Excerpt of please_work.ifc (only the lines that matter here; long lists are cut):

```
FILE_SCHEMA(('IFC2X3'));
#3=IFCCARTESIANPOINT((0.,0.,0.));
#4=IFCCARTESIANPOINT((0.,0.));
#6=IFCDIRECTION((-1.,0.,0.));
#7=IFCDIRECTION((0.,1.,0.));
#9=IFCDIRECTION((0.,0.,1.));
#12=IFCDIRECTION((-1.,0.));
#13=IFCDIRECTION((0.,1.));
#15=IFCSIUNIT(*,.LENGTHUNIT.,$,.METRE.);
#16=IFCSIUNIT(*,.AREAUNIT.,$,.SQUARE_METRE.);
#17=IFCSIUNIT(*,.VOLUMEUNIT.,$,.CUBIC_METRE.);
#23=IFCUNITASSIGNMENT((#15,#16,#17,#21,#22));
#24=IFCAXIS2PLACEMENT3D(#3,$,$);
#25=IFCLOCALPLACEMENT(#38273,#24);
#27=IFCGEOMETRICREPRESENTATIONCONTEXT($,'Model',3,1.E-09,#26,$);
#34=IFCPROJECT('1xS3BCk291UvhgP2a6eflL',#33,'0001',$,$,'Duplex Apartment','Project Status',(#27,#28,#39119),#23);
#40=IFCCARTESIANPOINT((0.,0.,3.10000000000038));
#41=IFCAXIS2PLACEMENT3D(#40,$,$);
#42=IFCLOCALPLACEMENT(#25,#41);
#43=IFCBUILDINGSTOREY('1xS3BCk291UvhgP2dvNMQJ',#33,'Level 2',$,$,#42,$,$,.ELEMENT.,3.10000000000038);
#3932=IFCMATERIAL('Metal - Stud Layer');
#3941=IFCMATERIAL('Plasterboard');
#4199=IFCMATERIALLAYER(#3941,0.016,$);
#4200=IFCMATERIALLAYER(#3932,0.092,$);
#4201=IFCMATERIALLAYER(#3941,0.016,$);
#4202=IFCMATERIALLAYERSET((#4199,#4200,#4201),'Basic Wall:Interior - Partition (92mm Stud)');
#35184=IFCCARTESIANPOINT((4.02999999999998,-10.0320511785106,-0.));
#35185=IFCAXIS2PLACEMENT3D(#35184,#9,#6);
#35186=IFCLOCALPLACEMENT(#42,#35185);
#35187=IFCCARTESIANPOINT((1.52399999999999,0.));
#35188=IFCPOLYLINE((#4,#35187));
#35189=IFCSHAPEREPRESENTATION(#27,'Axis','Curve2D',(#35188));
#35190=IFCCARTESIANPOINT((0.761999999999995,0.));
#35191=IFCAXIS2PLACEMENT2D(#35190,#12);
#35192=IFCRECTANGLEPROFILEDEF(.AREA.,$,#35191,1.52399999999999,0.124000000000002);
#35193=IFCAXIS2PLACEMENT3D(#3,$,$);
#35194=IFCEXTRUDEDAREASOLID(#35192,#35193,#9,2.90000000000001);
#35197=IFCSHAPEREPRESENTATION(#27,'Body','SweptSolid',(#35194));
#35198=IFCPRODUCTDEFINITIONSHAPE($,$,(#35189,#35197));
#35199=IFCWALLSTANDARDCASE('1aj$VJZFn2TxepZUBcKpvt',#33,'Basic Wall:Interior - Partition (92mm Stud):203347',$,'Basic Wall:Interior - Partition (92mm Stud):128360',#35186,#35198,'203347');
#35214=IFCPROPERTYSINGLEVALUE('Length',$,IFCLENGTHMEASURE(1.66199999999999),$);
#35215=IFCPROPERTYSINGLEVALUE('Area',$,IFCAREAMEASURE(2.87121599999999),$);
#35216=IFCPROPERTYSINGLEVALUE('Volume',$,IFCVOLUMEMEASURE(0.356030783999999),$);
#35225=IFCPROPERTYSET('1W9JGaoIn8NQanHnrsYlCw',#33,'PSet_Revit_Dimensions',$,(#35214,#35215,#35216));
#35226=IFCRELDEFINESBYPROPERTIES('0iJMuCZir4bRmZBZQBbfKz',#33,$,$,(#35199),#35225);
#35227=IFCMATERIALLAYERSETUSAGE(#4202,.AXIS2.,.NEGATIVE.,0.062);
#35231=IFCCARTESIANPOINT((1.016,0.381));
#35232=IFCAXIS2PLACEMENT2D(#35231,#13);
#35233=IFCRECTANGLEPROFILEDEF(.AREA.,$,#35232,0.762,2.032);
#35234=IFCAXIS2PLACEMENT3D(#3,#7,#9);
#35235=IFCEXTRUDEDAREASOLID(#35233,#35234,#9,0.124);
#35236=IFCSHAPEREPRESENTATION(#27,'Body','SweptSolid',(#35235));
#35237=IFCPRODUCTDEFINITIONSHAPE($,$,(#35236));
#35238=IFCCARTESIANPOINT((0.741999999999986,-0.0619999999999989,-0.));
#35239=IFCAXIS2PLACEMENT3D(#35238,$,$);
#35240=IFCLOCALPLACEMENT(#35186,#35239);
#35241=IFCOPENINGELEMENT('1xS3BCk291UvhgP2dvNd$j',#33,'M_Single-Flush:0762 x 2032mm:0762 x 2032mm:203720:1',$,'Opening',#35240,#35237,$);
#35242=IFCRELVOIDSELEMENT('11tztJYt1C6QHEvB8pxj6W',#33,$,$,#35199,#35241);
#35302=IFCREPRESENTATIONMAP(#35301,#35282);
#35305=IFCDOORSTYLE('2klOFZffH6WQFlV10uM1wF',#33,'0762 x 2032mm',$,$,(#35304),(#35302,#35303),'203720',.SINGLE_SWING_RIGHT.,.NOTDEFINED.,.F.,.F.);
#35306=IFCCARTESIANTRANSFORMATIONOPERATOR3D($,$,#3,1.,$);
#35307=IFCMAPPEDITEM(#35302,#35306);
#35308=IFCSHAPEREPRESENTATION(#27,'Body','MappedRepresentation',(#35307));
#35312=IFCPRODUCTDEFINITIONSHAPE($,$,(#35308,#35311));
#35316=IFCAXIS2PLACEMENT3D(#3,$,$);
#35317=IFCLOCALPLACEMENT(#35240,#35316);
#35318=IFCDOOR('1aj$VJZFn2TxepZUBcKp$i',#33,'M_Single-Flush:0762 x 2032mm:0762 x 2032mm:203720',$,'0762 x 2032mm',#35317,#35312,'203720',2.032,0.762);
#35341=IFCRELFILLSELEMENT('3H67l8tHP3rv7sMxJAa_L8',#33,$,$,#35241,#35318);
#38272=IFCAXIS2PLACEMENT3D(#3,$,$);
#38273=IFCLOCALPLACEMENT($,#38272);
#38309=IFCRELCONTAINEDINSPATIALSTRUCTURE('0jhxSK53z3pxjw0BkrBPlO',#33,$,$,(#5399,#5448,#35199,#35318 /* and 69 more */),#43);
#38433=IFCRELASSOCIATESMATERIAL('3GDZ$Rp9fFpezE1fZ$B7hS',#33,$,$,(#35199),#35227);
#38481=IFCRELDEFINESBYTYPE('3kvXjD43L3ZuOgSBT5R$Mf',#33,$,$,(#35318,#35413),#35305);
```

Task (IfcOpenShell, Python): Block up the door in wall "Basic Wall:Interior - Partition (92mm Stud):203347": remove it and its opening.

```python
import ifcopenshell
import ifcopenshell.api.feature
import ifcopenshell.api.pset
import ifcopenshell.api.root
import ifcopenshell.geom
import ifcopenshell.util.element
import ifcopenshell.util.shape
import ifcopenshell.util.unit

model = ifcopenshell.open("please_work.ifc")
area_scale = ifcopenshell.util.unit.calculate_unit_scale(model, "AREAUNIT")
volume_scale = ifcopenshell.util.unit.calculate_unit_scale(model, "VOLUMEUNIT")
settings = ifcopenshell.geom.settings()


def volume(element):
    """Net volume in cubic metres, openings subtracted."""
    shape = ifcopenshell.geom.create_shape(settings, element)
    return ifcopenshell.util.shape.get_volume(shape.geometry)


door = model.by_guid("1aj$VJZFn2TxepZUBcKp$i")
opening = door.FillsVoids[0].RelatingOpeningElement
wall = opening.VoidsElements[0].RelatingBuildingElement
before = volume(wall)

ifcopenshell.api.root.remove_product(model, product=door)
ifcopenshell.api.feature.remove_feature(model, feature=opening)

after = volume(wall)
thickness = 0.124  # wall thickness in metres

# Update the wall's stored quantities.
pset = model.by_id(ifcopenshell.util.element.get_pset(wall, "PSet_Revit_Dimensions", should_inherit=False)["id"])
ifcopenshell.api.pset.edit_pset(model, pset=pset, properties={
    "Area": model.create_entity("IfcAreaMeasure", after / thickness / area_scale),
    "Volume": model.create_entity("IfcVolumeMeasure", after / volume_scale),
})

print(f"wall volume {before:.3f} -> {after:.3f} m3")

model.write("please_work_rev.ifc")
```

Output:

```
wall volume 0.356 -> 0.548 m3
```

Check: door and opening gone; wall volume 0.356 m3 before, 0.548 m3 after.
